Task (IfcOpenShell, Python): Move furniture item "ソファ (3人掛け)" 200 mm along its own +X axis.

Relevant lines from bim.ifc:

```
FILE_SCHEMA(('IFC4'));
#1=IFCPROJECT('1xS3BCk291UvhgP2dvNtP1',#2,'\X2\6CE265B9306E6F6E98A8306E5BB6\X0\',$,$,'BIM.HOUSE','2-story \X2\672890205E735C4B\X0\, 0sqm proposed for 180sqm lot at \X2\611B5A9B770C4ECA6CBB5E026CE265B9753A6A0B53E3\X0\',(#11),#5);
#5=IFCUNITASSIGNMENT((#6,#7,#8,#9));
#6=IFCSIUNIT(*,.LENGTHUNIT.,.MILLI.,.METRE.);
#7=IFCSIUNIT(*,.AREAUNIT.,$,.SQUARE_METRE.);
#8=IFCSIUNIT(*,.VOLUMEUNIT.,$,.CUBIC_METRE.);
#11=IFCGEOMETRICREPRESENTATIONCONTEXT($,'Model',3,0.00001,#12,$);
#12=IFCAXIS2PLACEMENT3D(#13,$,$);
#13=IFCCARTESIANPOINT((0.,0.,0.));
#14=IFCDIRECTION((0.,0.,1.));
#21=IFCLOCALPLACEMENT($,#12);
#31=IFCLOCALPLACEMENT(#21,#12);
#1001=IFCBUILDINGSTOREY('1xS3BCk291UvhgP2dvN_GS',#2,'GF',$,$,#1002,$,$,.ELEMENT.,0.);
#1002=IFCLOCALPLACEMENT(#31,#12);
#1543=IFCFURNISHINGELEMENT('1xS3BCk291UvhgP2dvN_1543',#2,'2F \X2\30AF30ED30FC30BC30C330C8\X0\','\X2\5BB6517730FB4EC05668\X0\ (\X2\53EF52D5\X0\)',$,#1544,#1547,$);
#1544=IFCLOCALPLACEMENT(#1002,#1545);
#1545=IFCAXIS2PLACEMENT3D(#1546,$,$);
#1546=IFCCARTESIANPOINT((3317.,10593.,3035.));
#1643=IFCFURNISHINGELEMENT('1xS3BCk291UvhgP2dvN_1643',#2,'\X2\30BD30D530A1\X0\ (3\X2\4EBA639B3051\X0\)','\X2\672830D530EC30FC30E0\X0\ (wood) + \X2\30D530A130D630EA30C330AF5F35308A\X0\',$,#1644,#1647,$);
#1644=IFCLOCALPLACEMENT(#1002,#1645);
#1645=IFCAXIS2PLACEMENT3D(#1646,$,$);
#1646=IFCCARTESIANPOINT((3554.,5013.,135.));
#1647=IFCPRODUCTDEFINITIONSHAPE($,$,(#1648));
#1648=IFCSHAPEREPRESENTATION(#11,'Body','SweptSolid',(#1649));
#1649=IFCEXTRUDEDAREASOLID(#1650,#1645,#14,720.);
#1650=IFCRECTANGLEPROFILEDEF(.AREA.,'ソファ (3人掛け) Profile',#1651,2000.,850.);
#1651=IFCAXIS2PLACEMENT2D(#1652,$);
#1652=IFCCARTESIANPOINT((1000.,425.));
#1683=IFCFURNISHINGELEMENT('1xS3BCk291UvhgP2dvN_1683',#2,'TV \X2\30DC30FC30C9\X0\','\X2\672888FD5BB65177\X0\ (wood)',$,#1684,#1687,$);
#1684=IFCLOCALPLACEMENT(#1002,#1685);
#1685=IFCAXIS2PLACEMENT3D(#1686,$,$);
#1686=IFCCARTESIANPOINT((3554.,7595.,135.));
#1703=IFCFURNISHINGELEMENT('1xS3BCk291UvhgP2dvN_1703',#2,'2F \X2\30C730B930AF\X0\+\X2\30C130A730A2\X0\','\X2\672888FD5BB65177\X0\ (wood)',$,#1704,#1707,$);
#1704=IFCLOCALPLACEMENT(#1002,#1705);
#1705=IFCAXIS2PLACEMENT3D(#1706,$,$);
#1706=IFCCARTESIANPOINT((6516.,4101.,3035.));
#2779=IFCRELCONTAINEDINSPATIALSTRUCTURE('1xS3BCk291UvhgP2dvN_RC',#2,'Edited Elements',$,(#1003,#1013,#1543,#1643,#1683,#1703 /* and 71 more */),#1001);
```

```python
import ifcopenshell
import ifcopenshell.api.geometry
import ifcopenshell.util.placement
import ifcopenshell.util.unit

model = ifcopenshell.open("bim.ifc")
unit_scale = ifcopenshell.util.unit.calculate_unit_scale(model)

item = model.by_id(1643)
matrix = ifcopenshell.util.placement.get_local_placement(item.ObjectPlacement)
matrix[:3, 3] += matrix[:3, 0] * 0.2 / unit_scale
ifcopenshell.api.geometry.edit_object_placement(model, product=item, matrix=matrix, is_si=False)

print(ifcopenshell.util.placement.get_local_placement(item.ObjectPlacement).round(3) + 0.0)

model.write("bim-out.ifc")
```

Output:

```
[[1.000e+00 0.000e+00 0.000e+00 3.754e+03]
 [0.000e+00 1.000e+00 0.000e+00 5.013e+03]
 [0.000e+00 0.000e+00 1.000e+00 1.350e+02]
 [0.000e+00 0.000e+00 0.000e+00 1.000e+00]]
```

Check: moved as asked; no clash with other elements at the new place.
